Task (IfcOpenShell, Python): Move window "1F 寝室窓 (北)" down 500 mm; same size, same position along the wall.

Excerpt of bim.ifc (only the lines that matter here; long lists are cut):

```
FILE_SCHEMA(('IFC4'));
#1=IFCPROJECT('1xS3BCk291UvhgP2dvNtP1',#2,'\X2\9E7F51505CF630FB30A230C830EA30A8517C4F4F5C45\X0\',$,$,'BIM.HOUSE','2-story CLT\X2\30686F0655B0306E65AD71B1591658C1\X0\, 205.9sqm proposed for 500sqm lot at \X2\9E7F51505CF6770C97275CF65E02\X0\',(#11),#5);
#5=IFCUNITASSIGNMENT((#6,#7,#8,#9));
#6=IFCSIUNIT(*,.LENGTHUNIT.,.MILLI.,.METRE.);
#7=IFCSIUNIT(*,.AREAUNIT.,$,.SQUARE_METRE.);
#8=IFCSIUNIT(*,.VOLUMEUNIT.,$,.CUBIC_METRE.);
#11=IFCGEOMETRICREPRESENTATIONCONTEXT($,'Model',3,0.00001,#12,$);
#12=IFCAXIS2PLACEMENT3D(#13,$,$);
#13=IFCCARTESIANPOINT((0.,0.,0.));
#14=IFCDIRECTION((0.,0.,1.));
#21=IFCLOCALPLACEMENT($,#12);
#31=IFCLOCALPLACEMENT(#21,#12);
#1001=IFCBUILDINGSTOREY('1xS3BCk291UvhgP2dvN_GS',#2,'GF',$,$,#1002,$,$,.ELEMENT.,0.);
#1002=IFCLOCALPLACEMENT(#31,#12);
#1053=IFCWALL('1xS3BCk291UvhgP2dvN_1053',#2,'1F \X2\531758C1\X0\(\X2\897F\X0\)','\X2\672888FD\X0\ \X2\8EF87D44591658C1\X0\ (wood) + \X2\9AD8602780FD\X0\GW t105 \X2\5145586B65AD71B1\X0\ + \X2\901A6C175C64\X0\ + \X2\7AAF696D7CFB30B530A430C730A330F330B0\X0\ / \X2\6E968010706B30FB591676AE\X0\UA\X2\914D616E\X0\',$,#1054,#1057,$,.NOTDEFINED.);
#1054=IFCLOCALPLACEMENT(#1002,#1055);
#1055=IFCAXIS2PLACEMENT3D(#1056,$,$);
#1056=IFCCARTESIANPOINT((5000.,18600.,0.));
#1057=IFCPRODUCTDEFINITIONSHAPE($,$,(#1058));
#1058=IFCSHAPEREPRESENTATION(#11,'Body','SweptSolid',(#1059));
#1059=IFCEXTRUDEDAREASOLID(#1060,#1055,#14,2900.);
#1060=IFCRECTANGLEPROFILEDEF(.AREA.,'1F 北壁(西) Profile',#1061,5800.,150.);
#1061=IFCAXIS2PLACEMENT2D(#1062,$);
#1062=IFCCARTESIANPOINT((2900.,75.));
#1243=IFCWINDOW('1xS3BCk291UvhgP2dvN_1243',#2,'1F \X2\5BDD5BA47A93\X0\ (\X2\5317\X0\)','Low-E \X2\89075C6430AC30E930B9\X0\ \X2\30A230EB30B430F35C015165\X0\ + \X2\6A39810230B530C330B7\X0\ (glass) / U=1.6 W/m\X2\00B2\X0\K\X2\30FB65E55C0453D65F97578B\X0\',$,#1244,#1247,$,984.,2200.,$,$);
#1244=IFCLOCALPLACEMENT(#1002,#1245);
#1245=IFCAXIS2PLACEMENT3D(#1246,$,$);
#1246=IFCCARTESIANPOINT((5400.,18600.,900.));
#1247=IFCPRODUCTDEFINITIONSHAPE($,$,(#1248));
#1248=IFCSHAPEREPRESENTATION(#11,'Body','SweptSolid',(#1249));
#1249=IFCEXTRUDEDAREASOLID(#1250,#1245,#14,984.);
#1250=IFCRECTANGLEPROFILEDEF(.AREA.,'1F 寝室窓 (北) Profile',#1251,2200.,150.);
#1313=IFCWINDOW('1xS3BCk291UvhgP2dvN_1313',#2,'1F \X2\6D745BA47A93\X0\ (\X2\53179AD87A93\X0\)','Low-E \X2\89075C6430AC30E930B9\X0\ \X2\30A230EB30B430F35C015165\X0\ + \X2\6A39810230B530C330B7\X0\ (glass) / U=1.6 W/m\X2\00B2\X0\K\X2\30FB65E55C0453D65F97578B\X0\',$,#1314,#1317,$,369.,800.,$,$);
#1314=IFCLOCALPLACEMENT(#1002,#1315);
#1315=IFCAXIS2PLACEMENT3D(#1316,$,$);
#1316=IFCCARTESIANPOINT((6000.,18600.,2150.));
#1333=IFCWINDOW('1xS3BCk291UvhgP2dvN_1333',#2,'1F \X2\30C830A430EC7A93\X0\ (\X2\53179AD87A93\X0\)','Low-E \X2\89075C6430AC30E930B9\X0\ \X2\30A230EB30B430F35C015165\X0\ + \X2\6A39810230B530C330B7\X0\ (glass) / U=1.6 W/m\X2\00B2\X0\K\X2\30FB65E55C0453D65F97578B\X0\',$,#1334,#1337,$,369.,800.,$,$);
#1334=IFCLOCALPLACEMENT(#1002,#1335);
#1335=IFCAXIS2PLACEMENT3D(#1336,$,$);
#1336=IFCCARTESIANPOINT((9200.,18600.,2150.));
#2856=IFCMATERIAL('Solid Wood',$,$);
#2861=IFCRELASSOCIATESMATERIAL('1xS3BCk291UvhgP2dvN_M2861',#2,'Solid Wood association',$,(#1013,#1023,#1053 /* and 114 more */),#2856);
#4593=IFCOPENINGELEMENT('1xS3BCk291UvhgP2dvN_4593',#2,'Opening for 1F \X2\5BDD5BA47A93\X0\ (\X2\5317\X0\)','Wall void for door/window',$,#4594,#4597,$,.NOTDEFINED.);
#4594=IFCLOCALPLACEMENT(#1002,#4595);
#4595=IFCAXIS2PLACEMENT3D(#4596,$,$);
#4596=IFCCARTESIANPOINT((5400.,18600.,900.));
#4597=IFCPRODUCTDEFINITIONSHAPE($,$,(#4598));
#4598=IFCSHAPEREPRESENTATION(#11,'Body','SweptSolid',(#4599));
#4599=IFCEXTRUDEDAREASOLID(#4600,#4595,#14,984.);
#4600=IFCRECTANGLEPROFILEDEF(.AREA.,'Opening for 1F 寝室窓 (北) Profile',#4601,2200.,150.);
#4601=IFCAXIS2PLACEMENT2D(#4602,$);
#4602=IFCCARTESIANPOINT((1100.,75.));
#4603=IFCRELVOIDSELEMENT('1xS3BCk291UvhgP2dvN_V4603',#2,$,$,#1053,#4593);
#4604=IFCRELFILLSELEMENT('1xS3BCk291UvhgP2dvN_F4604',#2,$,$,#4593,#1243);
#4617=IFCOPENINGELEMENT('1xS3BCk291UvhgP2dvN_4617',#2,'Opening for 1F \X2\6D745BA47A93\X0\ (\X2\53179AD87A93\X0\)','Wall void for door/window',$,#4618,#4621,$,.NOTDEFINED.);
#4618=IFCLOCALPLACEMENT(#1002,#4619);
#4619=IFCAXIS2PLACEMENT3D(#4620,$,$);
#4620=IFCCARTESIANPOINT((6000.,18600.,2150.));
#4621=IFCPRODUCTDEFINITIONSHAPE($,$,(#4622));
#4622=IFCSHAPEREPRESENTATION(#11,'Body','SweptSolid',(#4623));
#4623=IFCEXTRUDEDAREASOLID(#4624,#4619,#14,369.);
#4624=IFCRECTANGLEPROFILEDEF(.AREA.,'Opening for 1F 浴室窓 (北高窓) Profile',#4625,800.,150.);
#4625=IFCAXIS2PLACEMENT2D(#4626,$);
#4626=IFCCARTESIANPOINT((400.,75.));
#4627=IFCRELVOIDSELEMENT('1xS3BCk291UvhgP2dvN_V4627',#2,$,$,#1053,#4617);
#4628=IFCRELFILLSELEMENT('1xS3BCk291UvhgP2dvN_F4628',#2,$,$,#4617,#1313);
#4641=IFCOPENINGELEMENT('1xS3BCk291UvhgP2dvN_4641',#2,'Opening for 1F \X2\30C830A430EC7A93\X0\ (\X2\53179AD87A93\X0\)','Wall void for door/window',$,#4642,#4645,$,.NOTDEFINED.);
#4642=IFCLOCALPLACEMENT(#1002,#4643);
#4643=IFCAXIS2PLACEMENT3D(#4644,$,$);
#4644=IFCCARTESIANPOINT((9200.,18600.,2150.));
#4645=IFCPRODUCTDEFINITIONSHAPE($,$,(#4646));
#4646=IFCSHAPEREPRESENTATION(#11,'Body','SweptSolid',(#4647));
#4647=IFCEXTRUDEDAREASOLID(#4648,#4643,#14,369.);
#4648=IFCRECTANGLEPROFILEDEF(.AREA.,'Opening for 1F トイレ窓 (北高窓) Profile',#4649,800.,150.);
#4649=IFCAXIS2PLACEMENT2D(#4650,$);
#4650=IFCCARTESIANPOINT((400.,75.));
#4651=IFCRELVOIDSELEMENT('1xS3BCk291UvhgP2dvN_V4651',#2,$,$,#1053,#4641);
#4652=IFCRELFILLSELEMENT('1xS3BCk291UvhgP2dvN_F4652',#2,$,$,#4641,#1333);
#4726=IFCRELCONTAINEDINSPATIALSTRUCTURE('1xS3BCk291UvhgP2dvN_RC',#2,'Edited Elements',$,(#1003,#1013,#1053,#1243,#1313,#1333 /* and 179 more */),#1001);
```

```python
import numpy as np
import ifcopenshell
import ifcopenshell.api.geometry
import ifcopenshell.util.placement
import ifcopenshell.util.unit

model = ifcopenshell.open("bim.ifc")
unit_scale = ifcopenshell.util.unit.calculate_unit_scale(model)

window = model.by_id(1243)
opening = window.FillsVoids[0].RelatingOpeningElement
dz = -0.5 / unit_scale

shift = np.array([0.0, 0.0, dz])
# The window is not placed relative to its opening, so move both.
for product in (opening, window):
    matrix = ifcopenshell.util.placement.get_local_placement(product.ObjectPlacement)
    matrix[:3, 3] += shift
    ifcopenshell.api.geometry.edit_object_placement(model, product=product, matrix=matrix, is_si=False)

print(f"moved by {dz * unit_scale:+.3f} m")

model.write("bim_rev.ifc")
```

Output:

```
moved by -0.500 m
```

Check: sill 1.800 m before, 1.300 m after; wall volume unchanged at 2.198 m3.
